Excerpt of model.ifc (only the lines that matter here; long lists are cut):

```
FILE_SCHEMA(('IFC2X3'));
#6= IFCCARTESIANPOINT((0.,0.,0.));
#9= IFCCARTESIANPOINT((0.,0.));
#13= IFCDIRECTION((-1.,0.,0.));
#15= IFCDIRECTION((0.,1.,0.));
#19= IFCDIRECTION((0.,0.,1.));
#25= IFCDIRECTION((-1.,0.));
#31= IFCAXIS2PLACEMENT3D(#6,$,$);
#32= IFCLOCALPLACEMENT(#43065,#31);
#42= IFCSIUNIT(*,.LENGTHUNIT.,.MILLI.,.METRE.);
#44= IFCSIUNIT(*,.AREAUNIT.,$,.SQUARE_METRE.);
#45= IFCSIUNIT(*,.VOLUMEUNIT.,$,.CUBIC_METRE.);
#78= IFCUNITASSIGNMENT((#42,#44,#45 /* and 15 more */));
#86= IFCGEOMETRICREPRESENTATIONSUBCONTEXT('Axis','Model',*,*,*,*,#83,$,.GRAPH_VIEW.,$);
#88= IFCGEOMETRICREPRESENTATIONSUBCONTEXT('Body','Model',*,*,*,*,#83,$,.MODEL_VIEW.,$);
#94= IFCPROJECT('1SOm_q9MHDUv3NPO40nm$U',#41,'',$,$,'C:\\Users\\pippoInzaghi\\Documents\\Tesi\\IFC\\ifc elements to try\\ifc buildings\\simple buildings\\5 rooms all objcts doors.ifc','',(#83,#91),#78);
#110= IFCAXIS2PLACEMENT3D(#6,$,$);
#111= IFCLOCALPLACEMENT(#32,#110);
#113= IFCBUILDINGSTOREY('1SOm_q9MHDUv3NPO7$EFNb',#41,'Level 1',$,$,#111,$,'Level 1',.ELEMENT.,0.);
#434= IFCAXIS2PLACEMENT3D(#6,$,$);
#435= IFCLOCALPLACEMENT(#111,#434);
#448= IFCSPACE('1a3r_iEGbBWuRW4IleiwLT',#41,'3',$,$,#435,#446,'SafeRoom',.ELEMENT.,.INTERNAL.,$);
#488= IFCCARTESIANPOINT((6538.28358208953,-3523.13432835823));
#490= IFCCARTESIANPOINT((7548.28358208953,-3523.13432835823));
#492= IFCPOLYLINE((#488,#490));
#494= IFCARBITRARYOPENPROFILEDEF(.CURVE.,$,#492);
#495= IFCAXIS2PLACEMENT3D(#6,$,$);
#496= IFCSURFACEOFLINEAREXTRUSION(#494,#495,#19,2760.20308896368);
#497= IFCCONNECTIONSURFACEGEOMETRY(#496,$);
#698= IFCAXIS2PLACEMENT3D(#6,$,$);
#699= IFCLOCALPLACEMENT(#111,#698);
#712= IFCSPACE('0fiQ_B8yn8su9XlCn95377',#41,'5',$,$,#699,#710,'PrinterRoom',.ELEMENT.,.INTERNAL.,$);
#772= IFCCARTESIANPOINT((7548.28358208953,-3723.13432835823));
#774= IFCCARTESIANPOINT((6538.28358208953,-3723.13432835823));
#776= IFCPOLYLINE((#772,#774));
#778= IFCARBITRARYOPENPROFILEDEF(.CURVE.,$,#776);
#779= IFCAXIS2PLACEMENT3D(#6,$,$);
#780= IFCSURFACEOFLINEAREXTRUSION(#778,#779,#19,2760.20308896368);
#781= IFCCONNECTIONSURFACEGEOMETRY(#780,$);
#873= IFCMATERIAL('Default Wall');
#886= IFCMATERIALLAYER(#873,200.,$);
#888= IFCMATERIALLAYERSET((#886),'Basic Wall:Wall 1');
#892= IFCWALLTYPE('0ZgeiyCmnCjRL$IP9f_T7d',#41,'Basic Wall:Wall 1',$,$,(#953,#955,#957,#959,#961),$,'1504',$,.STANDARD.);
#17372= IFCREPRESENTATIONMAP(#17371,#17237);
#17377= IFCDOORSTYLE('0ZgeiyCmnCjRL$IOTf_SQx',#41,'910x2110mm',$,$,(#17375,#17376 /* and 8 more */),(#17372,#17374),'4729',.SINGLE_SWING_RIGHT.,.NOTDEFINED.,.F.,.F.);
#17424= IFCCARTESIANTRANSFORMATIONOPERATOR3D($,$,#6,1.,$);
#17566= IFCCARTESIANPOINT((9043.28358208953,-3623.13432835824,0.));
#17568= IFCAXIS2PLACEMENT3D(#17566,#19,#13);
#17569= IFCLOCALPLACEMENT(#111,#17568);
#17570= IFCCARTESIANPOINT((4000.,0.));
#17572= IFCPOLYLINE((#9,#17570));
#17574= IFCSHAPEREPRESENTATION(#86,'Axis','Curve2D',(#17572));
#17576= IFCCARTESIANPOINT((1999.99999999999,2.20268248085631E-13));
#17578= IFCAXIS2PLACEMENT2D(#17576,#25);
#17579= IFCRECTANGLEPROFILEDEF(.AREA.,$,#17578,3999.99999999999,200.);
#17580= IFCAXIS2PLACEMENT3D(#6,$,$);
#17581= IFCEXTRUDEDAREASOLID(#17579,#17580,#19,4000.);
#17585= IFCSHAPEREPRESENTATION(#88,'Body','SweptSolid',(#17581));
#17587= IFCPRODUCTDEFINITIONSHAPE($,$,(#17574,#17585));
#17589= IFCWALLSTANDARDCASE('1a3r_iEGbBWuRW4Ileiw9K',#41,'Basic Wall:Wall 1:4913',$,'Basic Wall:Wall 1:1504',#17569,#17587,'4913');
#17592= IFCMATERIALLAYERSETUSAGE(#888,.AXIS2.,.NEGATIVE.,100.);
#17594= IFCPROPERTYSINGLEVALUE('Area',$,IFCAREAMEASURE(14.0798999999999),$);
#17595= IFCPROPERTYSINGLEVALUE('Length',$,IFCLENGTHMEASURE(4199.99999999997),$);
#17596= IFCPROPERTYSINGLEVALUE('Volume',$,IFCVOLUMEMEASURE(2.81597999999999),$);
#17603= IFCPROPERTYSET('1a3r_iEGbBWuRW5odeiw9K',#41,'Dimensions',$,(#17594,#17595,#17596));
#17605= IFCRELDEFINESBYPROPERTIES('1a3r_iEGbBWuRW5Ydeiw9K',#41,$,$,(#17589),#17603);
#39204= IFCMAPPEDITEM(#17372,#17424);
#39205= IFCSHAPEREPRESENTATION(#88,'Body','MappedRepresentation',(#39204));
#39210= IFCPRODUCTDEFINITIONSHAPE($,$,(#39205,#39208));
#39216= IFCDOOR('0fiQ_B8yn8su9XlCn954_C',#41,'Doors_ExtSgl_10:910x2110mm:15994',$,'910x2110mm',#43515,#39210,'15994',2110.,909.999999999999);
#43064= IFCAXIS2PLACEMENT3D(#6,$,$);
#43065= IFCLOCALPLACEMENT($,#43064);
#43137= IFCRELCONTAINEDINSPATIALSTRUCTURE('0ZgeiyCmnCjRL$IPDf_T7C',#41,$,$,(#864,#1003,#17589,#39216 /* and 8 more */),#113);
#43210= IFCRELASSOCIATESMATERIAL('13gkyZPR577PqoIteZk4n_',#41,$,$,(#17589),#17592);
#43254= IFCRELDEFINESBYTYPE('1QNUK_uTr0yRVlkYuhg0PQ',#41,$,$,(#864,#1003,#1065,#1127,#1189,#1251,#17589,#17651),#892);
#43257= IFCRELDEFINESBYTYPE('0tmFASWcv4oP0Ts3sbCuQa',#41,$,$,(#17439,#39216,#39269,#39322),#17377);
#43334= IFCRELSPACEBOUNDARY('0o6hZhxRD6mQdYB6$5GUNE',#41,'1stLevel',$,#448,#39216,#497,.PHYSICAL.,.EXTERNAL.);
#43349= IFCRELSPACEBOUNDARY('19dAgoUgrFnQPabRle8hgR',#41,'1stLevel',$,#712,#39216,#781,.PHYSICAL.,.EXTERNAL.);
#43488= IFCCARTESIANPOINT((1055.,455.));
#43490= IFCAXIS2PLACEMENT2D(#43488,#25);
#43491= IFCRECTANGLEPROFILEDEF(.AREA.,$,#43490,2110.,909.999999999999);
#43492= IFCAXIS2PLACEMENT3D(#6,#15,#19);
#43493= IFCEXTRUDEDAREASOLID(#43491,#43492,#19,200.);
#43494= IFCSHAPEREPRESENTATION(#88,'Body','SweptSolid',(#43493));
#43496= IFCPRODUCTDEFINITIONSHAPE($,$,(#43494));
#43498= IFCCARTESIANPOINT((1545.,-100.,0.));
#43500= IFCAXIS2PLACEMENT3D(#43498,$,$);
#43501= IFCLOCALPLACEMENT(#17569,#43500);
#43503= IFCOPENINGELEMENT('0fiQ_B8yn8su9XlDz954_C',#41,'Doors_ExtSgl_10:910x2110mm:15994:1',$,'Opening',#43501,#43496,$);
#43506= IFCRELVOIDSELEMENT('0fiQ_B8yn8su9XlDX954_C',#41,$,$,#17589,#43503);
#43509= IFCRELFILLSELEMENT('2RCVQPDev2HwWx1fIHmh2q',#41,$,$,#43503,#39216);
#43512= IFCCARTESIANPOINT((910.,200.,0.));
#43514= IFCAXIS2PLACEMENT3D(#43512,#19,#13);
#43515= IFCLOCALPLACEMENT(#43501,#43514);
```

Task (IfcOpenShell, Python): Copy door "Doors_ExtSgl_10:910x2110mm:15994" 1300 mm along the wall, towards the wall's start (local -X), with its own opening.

```python
import numpy as np
import ifcopenshell
import ifcopenshell.api.feature
import ifcopenshell.api.geometry
import ifcopenshell.api.pset
import ifcopenshell.api.root
import ifcopenshell.geom
import ifcopenshell.util.element
import ifcopenshell.util.placement
import ifcopenshell.util.shape
import ifcopenshell.util.unit

model = ifcopenshell.open("model.ifc")
unit_scale = ifcopenshell.util.unit.calculate_unit_scale(model)
area_scale = ifcopenshell.util.unit.calculate_unit_scale(model, "AREAUNIT")
volume_scale = ifcopenshell.util.unit.calculate_unit_scale(model, "VOLUMEUNIT")
settings = ifcopenshell.geom.settings()


def volume(element):
    """Net volume in cubic metres, openings subtracted."""
    shape = ifcopenshell.geom.create_shape(settings, element)
    return ifcopenshell.util.shape.get_volume(shape.geometry)


def reuse_history(source, copy):
    """copy_class also copies each property set's owner history, people and application; keep the originals."""
    for rel in copy.IsDefinedBy:
        if rel.is_a("IfcRelDefinesByProperties") and (history := rel.RelatingPropertyDefinition.OwnerHistory):
            rel.RelatingPropertyDefinition.OwnerHistory = source.OwnerHistory
            ifcopenshell.util.element.remove_deep2(model, history)


door = model.by_id(39216)
opening = door.FillsVoids[0].RelatingOpeningElement
wall = opening.VoidsElements[0].RelatingBuildingElement
before = volume(wall)
shift = ifcopenshell.util.placement.get_local_placement(wall.ObjectPlacement)[:3, 0] * -1.3 / unit_scale

# copy_class copies the void relationship, type, container and properties, but no geometry.
new_opening = ifcopenshell.api.root.copy_class(model, product=opening)
new_opening.Representation = ifcopenshell.util.element.copy_deep(
    model, opening.Representation, exclude=["IfcGeometricRepresentationContext", "IfcRepresentationMap"]
)
new_opening.Name = "Doors_ExtSgl_10:910x2110mm"
new_door = ifcopenshell.api.root.copy_class(model, product=door)
new_door.Representation = ifcopenshell.util.element.copy_deep(
    model, door.Representation, exclude=["IfcGeometricRepresentationContext", "IfcRepresentationMap"]
)
new_door.Name = "Doors_ExtSgl_10:910x2110mm"
new_door.Tag = None
reuse_history(door, new_door)
fills = ifcopenshell.api.feature.add_filling(model, opening=new_opening, element=new_door)
fills.OwnerHistory = new_door.OwnerHistory  # required in IFC2X3

for old, new in ((opening, new_opening), (door, new_door)):
    matrix = ifcopenshell.util.placement.get_local_placement(old.ObjectPlacement)
    matrix[:3, 3] += shift
    ifcopenshell.api.geometry.edit_object_placement(model, product=new, matrix=matrix, is_si=False)

# The copied space boundaries still share their surfaces with the original.
for rel in new_door.ProvidesBoundaries:
    if rel.ConnectionGeometry:
        rel.ConnectionGeometry = ifcopenshell.util.element.copy_deep(model, rel.ConnectionGeometry)

# Space boundary surfaces are stored in each space's coordinates; move them too.
for rel in new_door.ProvidesBoundaries:
    if not rel.ConnectionGeometry:
        continue
    surface = rel.ConnectionGeometry.SurfaceOnRelatingElement
    space_matrix = ifcopenshell.util.placement.get_local_placement(rel.RelatingSpace.ObjectPlacement)
    point = np.array(surface.Position.Location.Coordinates) + space_matrix[:3, :3].T @ shift
    surface.Position = model.createIfcAxis2Placement3D(
        model.createIfcCartesianPoint(point.tolist()), surface.Position.Axis, surface.Position.RefDirection
    )

after = volume(wall)
thickness = 0.2  # wall thickness in metres

# Update the wall's stored quantities.
pset = model.by_id(ifcopenshell.util.element.get_pset(wall, "Dimensions", should_inherit=False)["id"])
ifcopenshell.api.pset.edit_pset(model, pset=pset, properties={
    "Area": model.create_entity("IfcAreaMeasure", after / thickness / area_scale),
    "Volume": model.create_entity("IfcVolumeMeasure", after / volume_scale),
})

print(f"wall volume {before:.3f} -> {after:.3f} m3")

model.write("model_edited.ifc")
```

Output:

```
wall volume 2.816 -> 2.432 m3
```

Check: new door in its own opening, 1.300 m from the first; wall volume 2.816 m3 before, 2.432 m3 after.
